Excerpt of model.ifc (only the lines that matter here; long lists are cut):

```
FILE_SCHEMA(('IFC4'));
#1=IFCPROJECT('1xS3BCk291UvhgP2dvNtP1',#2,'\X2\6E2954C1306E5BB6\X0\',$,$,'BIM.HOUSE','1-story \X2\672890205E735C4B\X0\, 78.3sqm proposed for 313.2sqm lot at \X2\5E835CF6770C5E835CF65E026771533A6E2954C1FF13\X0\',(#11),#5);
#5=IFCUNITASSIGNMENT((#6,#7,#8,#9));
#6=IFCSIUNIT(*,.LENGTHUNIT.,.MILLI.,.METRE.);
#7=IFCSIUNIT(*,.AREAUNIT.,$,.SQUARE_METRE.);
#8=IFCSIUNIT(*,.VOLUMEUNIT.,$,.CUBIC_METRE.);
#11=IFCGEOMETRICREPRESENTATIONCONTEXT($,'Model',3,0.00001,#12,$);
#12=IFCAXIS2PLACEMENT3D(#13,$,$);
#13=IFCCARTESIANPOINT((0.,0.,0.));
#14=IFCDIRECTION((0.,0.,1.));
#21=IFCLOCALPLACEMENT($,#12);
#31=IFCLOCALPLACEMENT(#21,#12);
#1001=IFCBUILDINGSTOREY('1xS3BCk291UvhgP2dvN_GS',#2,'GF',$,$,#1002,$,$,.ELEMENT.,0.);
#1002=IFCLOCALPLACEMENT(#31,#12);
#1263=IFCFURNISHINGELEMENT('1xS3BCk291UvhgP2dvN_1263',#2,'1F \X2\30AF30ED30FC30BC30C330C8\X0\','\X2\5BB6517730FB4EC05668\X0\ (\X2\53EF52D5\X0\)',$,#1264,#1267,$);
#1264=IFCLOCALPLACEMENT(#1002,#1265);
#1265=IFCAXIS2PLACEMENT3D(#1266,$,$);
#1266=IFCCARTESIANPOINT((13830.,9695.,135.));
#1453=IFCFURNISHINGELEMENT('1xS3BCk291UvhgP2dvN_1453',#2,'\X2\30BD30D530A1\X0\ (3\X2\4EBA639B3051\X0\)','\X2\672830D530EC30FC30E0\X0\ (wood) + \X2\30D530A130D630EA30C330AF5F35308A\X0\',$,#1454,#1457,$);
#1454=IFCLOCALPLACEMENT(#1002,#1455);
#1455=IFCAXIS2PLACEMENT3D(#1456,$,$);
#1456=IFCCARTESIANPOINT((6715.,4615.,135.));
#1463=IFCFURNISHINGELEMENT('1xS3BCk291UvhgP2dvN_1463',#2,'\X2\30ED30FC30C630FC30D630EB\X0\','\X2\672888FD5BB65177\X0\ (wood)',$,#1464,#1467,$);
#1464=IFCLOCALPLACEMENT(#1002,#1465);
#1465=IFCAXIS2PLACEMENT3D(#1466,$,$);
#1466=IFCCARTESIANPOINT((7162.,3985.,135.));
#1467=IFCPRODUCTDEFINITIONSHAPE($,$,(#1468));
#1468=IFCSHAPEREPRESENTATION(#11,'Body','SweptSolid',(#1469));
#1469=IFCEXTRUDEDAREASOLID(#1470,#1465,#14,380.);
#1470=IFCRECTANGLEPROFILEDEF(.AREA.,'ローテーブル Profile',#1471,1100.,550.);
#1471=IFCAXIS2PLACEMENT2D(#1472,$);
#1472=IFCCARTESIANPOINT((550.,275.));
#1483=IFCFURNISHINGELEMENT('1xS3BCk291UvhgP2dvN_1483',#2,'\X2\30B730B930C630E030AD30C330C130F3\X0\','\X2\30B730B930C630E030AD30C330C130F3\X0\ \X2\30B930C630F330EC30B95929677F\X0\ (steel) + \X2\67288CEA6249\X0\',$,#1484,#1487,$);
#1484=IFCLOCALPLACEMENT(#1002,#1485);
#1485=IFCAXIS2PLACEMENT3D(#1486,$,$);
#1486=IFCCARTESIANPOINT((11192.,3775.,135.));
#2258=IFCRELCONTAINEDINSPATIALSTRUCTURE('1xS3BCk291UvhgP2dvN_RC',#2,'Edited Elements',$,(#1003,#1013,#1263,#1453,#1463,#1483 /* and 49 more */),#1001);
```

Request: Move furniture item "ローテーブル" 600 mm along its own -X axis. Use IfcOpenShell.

```python
import ifcopenshell
import ifcopenshell.api.geometry
import ifcopenshell.util.placement

model = ifcopenshell.open("model.ifc")

item = model.by_guid("1xS3BCk291UvhgP2dvN_1463")
matrix = ifcopenshell.util.placement.get_local_placement(item.ObjectPlacement)
matrix[:3, 3] -= matrix[:3, 0] * 600.0
ifcopenshell.api.geometry.edit_object_placement(model, product=item, matrix=matrix, is_si=False)

print(ifcopenshell.util.placement.get_local_placement(item.ObjectPlacement).round(3) + 0.0)

model.write("model_edited.ifc")
```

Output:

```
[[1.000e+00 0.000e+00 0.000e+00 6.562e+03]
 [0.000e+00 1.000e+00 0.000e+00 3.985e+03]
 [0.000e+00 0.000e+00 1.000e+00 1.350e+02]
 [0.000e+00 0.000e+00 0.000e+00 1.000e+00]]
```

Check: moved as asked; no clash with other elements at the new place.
